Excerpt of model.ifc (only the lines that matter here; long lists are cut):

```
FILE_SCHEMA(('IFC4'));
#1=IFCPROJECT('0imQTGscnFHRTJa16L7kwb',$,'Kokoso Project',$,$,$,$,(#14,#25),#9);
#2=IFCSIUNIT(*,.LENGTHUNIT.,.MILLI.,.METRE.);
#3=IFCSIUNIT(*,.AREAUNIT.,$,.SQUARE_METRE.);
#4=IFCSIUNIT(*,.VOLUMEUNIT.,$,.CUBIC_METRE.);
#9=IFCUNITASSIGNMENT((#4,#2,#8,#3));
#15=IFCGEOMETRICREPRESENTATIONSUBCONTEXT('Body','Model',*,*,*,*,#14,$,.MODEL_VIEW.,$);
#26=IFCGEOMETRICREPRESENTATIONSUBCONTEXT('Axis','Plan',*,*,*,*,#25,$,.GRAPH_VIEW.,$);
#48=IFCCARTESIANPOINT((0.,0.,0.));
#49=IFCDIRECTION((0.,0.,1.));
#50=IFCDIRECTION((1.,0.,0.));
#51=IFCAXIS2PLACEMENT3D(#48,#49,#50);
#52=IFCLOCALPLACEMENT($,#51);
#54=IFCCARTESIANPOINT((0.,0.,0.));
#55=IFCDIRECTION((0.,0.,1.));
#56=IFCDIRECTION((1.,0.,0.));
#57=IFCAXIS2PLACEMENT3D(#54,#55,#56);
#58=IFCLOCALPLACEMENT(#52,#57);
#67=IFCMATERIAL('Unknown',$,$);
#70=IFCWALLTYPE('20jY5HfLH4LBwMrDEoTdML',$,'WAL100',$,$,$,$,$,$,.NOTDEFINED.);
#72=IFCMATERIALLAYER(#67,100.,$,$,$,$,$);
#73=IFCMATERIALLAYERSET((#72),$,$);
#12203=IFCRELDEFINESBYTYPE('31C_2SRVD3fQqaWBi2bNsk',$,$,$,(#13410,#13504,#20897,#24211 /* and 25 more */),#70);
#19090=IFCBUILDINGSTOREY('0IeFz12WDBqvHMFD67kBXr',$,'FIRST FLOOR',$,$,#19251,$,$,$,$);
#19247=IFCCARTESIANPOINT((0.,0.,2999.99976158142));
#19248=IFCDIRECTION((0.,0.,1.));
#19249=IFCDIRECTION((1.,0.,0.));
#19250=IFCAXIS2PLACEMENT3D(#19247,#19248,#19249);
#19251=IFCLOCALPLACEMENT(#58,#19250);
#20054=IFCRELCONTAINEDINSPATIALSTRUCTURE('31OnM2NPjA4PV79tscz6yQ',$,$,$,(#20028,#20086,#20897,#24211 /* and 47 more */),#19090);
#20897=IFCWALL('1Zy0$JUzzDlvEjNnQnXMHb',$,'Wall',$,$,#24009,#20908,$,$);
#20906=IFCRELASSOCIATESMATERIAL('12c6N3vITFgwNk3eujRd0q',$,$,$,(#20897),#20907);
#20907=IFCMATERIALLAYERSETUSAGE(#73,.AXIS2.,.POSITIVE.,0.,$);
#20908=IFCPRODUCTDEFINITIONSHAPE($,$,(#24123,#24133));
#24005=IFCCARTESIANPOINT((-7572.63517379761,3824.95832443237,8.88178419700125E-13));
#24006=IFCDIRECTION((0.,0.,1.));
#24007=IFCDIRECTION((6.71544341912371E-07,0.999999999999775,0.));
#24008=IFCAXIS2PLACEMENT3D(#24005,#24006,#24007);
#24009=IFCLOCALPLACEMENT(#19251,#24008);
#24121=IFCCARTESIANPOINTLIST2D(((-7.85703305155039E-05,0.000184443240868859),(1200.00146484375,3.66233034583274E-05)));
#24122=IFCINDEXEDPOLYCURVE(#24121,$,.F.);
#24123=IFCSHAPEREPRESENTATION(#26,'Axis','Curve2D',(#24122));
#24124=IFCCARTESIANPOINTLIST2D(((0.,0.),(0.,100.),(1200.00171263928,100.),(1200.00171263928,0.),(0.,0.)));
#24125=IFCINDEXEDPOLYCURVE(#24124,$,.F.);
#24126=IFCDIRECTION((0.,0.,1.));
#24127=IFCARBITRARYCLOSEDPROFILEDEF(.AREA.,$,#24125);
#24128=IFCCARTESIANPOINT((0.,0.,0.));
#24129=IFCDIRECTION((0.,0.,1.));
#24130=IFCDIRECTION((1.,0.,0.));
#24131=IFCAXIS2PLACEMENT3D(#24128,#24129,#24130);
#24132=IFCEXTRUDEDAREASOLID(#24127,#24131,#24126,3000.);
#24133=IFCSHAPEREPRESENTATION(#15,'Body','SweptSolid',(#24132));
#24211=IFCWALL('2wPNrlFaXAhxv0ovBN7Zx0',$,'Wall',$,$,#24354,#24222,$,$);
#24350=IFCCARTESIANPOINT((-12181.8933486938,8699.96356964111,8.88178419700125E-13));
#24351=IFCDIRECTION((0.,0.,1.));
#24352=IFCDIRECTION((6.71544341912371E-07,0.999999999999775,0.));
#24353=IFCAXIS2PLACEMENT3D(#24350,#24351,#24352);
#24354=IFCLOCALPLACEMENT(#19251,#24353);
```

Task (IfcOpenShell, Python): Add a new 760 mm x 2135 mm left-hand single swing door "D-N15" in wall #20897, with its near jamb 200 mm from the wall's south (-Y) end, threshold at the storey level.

```python
import numpy as np
import ifcopenshell
import ifcopenshell.api.feature
import ifcopenshell.api.geometry
import ifcopenshell.api.root
import ifcopenshell.api.spatial
import ifcopenshell.geom
import ifcopenshell.util.element
import ifcopenshell.util.placement
import ifcopenshell.util.representation
import ifcopenshell.util.shape
import ifcopenshell.util.unit

model = ifcopenshell.open("model.ifc")
unit_scale = ifcopenshell.util.unit.calculate_unit_scale(model)
settings = ifcopenshell.geom.settings()


def volume(element):
    """Net volume in cubic metres, openings subtracted."""
    shape = ifcopenshell.geom.create_shape(settings, element)
    return ifcopenshell.util.shape.get_volume(shape.geometry)


wall = model.by_guid("1Zy0$JUzzDlvEjNnQnXMHb")
storey = ifcopenshell.util.element.get_container(wall, ifc_class="IfcBuildingStorey")
context = ifcopenshell.util.representation.get_context(model, "Model", "Body", "MODEL_VIEW")
before = volume(wall)

width, height, from_end, sill = 0.76, 2.135, 0.2, 0.0  # metres

# The wall runs along its own X axis, and the end named is its -X end.
wall_shape = ifcopenshell.geom.create_shape(settings, wall)
x, y, z = ifcopenshell.util.shape.get_vertices(wall_shape.geometry).T
start = x.min() + from_end
face, thickness = float(y.min()), float(y.max() - y.min())
wall_matrix = ifcopenshell.util.placement.get_local_placement(wall.ObjectPlacement)
level = ifcopenshell.util.placement.get_local_placement(storey.ObjectPlacement)[2, 3]


def in_wall(x, y):
    """Placement at x, y metres in the wall's axes, at sill height."""
    matrix = wall_matrix.copy()
    matrix[:, 3] = wall_matrix @ np.array([x / unit_scale, y / unit_scale, 0.0, 1.0])
    matrix[2, 3] = level + sill / unit_scale
    return matrix


# Opening: a box that overshoots both wall faces by 50 mm.
opening = ifcopenshell.api.root.create_entity(model, ifc_class="IfcOpeningElement", predefined_type="OPENING")
box = ifcopenshell.api.geometry.add_wall_representation(
    model, context=context, length=width, height=height, thickness=thickness + 0.1
)
ifcopenshell.api.geometry.assign_representation(model, product=opening, representation=box)
ifcopenshell.api.geometry.edit_object_placement(model, product=opening, matrix=in_wall(start, face - 0.05), is_si=False)
ifcopenshell.api.feature.add_feature(model, feature=opening, element=wall)

door = ifcopenshell.api.root.create_entity(model, ifc_class="IfcDoor", name="D-N15", predefined_type="DOOR")
door.OverallWidth, door.OverallHeight = width / unit_scale, height / unit_scale
door.OperationType = "SINGLE_SWING_LEFT"
body = ifcopenshell.api.geometry.add_door_representation(
    model,
    context=context,
    overall_width=door.OverallWidth,
    overall_height=door.OverallHeight,
    operation_type="SINGLE_SWING_LEFT",
    lining_properties={"LiningDepth": thickness / unit_scale, "ThresholdDepth": thickness / unit_scale},
)
ifcopenshell.api.geometry.assign_representation(model, product=door, representation=body)
ifcopenshell.api.spatial.assign_container(model, products=[door], relating_structure=storey)
ifcopenshell.api.feature.add_filling(model, opening=opening, element=door)

# The lining spans the wall, so the door starts at the wall face.
ifcopenshell.api.geometry.edit_object_placement(model, product=door, matrix=in_wall(start, face), is_si=False)

after = volume(wall)

print(f"wall volume {before:.3f} -> {after:.3f} m3")

model.write("model_v2.ifc")
```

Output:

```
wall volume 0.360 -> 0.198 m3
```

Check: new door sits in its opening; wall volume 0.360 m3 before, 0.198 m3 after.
